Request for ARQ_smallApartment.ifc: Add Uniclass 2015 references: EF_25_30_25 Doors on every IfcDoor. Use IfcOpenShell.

First a look at what the model holds.

```python
import ifcopenshell

model = ifcopenshell.open("ARQ_smallApartment.ifc")
print(model.schema)
print("classifications:", [c.Name for c in model.by_type("IfcClassification")])
for ifc_class in ("IfcDoor", "IfcRoof", "IfcStair", "IfcWall", "IfcWindow"):
    print(ifc_class, len(model.by_type(ifc_class)))
```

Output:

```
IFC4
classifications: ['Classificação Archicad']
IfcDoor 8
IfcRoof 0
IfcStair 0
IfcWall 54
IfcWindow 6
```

```python
import ifcopenshell
import ifcopenshell.api.classification

model = ifcopenshell.open("ARQ_smallApartment.ifc")

system = ifcopenshell.api.classification.add_classification(model, classification="Uniclass 2015")

codes = {
    "IfcDoor": ("EF_25_30_25", "Doors"),
}
for ifc_class, (code, name) in codes.items():
    products = model.by_type(ifc_class)
    ifcopenshell.api.classification.add_reference(
        model, products=products, classification=system, identification=code, name=name
    )
    print(code, len(products))

model.write("ARQ_smallApartment_updated.ifc")
```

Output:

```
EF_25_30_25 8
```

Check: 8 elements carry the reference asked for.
